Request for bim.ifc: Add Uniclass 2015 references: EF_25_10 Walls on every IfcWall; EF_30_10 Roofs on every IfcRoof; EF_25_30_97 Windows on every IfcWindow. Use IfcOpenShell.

First a look at what the model holds.

```python
import ifcopenshell

model = ifcopenshell.open("bim.ifc")
print(model.schema)
print("classifications:", [c.Name for c in model.by_type("IfcClassification")])
for ifc_class in ("IfcDoor", "IfcRoof", "IfcStair", "IfcWall", "IfcWindow"):
    print(ifc_class, len(model.by_type(ifc_class)))
```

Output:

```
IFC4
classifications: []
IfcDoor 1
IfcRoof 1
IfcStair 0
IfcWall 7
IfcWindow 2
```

```python
import ifcopenshell
import ifcopenshell.api.classification

model = ifcopenshell.open("bim.ifc")

system = ifcopenshell.api.classification.add_classification(model, classification="Uniclass 2015")

codes = {
    "IfcWall": ("EF_25_10", "Walls"),
    "IfcRoof": ("EF_30_10", "Roofs"),
    "IfcWindow": ("EF_25_30_97", "Windows"),
}
for ifc_class, (code, name) in codes.items():
    products = model.by_type(ifc_class)
    ifcopenshell.api.classification.add_reference(
        model, products=products, classification=system, identification=code, name=name
    )
    print(code, len(products))

model.write("bim_v2.ifc")
```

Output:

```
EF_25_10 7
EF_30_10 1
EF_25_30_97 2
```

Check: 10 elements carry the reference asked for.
